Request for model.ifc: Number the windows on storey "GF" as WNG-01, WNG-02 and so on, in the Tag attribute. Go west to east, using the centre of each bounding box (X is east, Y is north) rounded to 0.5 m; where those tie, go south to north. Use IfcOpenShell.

First a look at what the model holds.

```python
import ifcopenshell
import ifcopenshell.util.element
import ifcopenshell.util.placement

model = ifcopenshell.open("model.ifc")
print(model.schema)
storey = next(s for s in model.by_type("IfcBuildingStorey") if s.Name == "GF")
windows = [e for e in ifcopenshell.util.element.get_decomposition(storey) if e.is_a("IfcWindow")]
for e in sorted(windows, key=lambda e: e.id()):
    origin = ifcopenshell.util.placement.get_local_placement(e.ObjectPlacement)[:3, 3]
    print(e.id(), e.Tag, e.Name, origin.round(2) + 0.0, sep=" | ")
```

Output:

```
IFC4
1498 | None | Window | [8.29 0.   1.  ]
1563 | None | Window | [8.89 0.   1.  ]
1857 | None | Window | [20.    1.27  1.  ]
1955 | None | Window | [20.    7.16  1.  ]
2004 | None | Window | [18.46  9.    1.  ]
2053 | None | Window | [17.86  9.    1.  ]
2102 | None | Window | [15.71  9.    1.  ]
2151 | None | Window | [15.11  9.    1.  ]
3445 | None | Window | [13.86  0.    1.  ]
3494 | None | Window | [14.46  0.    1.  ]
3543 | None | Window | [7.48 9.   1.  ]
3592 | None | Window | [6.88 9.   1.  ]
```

```python
import ifcopenshell
import ifcopenshell.geom
import ifcopenshell.util.element
import ifcopenshell.util.shape

model = ifcopenshell.open("model.ifc")
settings = ifcopenshell.geom.settings()
settings.set("use-world-coords", True)


def centre(element):
    shape = ifcopenshell.geom.create_shape(settings, element)
    return ifcopenshell.util.shape.get_bbox_centroid(shape.geometry)


storey = next(s for s in model.by_type("IfcBuildingStorey") if s.Name == "GF")
windows = [e for e in ifcopenshell.util.element.get_decomposition(storey) if e.is_a("IfcWindow")]

# Insertion points can sit at a corner or the storey origin, so sort by the geometry (in metres).
centres = {e: centre(e) for e in windows}
windows.sort(key=lambda e: (round(centres[e][0] / 0.5), centres[e][1]))

for i, e in enumerate(windows, start=1):
    number = f"WNG-{i:02d}"
    e.Tag = number
    print(e.id(), number)

model.write("model_edited.ifc")
```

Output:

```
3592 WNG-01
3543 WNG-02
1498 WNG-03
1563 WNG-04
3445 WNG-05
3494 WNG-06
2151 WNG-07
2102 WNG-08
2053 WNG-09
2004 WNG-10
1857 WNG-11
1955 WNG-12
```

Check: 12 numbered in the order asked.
